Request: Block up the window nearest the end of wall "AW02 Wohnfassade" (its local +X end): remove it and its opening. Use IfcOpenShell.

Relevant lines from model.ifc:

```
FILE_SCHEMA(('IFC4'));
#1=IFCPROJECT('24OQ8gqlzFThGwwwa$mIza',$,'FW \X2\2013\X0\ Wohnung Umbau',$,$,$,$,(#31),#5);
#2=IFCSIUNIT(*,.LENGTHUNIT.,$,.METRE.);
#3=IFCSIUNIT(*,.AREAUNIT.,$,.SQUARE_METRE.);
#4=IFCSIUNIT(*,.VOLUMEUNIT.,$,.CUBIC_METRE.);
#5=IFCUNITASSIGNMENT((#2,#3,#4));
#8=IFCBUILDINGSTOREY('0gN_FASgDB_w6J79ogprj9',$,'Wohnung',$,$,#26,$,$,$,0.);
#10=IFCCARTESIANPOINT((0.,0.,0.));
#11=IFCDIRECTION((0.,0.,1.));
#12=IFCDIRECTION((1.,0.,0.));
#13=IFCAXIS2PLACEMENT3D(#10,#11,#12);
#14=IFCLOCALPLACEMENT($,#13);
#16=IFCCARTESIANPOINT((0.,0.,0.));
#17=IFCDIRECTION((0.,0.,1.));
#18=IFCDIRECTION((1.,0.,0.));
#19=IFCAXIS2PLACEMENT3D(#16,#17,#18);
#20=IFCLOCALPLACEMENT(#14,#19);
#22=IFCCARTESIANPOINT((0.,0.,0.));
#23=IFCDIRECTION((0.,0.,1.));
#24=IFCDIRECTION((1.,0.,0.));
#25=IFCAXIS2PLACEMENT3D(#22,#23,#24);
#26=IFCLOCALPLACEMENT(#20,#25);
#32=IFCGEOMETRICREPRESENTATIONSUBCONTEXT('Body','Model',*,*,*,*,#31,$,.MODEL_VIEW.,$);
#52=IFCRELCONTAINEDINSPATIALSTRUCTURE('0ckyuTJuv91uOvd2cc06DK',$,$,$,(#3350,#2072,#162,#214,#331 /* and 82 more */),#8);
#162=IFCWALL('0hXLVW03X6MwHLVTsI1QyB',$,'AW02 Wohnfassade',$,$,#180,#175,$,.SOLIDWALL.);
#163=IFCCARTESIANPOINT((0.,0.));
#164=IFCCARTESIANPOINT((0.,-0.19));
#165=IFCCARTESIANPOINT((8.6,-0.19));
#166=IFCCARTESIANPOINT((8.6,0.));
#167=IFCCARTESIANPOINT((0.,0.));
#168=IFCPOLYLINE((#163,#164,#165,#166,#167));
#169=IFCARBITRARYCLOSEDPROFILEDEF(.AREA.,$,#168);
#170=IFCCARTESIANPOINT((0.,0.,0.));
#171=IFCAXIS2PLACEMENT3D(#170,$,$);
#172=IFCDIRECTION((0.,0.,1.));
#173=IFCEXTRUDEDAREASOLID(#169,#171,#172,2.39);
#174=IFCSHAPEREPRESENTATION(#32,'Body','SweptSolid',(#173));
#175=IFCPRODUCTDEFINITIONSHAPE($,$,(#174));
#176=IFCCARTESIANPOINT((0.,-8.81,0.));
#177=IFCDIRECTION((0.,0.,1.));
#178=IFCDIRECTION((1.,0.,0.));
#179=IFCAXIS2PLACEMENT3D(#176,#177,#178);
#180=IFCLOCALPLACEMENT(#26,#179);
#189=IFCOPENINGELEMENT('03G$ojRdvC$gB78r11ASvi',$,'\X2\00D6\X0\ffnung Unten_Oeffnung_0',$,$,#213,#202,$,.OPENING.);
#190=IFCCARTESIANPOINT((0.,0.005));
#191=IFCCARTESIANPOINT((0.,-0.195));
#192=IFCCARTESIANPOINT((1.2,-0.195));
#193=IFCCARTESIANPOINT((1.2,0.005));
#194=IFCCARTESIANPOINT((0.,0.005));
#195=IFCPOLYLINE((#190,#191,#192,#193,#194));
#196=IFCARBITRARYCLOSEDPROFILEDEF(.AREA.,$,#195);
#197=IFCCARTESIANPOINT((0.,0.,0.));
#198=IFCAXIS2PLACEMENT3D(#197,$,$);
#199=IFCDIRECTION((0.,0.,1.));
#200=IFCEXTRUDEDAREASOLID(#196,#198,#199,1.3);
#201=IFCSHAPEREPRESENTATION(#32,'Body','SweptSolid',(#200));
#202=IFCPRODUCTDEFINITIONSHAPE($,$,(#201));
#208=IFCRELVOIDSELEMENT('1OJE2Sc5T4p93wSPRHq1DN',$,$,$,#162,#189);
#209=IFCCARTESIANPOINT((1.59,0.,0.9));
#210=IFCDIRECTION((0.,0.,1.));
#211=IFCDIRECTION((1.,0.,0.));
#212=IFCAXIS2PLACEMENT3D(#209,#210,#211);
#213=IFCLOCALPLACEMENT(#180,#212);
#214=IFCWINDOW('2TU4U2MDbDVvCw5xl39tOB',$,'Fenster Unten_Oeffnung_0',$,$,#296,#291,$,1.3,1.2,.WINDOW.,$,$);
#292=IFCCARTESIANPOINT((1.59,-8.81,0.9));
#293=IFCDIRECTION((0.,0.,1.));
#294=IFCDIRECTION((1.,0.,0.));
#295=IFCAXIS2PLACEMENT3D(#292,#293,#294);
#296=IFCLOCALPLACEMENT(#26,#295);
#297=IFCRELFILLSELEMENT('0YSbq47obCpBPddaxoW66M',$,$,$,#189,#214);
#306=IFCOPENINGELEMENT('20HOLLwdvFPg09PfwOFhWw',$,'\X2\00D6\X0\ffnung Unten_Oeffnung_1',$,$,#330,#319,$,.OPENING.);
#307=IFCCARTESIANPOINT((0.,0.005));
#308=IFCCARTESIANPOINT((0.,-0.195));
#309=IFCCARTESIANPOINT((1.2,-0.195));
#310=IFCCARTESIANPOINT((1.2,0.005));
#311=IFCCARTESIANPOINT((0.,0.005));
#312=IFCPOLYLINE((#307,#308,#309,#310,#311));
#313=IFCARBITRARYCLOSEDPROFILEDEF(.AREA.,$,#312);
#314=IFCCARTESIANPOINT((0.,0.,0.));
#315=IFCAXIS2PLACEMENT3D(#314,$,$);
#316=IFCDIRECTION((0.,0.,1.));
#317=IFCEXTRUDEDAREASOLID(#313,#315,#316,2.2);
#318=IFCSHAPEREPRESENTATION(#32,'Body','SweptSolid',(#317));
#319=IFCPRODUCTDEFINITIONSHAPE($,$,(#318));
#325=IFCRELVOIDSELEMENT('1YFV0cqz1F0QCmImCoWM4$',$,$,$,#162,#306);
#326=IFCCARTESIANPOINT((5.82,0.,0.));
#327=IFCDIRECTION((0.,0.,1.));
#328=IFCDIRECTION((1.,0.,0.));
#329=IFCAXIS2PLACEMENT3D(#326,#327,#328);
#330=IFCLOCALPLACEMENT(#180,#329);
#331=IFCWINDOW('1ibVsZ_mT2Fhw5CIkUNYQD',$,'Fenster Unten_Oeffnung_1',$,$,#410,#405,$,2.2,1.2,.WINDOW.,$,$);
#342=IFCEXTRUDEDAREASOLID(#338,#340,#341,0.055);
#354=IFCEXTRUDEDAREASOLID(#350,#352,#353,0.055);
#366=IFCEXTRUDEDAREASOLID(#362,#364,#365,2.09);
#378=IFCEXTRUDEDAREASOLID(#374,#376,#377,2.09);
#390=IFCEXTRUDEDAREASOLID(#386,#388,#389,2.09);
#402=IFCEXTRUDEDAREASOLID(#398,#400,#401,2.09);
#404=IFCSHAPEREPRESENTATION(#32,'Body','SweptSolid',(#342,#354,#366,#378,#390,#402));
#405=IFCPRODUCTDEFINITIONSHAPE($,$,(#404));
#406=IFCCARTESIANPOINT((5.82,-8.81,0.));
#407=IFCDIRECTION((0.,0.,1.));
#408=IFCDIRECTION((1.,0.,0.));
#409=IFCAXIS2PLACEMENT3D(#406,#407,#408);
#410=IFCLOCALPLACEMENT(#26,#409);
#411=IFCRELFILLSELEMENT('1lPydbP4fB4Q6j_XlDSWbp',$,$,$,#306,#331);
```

```python
import ifcopenshell
import ifcopenshell.api.feature
import ifcopenshell.api.root
import ifcopenshell.geom
import ifcopenshell.util.shape

model = ifcopenshell.open("model.ifc")
settings = ifcopenshell.geom.settings()


def volume(element):
    """Net volume in cubic metres, openings subtracted."""
    shape = ifcopenshell.geom.create_shape(settings, element)
    return ifcopenshell.util.shape.get_volume(shape.geometry)


window = model.by_guid("1ibVsZ_mT2Fhw5CIkUNYQD")
opening = window.FillsVoids[0].RelatingOpeningElement
wall = opening.VoidsElements[0].RelatingBuildingElement
before = volume(wall)

ifcopenshell.api.root.remove_product(model, product=window)
ifcopenshell.api.feature.remove_feature(model, feature=opening)

after = volume(wall)

print(f"wall volume {before:.3f} -> {after:.3f} m3")

model.write("model_updated.ifc")
```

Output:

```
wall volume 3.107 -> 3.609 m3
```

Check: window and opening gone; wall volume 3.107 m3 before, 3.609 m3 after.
